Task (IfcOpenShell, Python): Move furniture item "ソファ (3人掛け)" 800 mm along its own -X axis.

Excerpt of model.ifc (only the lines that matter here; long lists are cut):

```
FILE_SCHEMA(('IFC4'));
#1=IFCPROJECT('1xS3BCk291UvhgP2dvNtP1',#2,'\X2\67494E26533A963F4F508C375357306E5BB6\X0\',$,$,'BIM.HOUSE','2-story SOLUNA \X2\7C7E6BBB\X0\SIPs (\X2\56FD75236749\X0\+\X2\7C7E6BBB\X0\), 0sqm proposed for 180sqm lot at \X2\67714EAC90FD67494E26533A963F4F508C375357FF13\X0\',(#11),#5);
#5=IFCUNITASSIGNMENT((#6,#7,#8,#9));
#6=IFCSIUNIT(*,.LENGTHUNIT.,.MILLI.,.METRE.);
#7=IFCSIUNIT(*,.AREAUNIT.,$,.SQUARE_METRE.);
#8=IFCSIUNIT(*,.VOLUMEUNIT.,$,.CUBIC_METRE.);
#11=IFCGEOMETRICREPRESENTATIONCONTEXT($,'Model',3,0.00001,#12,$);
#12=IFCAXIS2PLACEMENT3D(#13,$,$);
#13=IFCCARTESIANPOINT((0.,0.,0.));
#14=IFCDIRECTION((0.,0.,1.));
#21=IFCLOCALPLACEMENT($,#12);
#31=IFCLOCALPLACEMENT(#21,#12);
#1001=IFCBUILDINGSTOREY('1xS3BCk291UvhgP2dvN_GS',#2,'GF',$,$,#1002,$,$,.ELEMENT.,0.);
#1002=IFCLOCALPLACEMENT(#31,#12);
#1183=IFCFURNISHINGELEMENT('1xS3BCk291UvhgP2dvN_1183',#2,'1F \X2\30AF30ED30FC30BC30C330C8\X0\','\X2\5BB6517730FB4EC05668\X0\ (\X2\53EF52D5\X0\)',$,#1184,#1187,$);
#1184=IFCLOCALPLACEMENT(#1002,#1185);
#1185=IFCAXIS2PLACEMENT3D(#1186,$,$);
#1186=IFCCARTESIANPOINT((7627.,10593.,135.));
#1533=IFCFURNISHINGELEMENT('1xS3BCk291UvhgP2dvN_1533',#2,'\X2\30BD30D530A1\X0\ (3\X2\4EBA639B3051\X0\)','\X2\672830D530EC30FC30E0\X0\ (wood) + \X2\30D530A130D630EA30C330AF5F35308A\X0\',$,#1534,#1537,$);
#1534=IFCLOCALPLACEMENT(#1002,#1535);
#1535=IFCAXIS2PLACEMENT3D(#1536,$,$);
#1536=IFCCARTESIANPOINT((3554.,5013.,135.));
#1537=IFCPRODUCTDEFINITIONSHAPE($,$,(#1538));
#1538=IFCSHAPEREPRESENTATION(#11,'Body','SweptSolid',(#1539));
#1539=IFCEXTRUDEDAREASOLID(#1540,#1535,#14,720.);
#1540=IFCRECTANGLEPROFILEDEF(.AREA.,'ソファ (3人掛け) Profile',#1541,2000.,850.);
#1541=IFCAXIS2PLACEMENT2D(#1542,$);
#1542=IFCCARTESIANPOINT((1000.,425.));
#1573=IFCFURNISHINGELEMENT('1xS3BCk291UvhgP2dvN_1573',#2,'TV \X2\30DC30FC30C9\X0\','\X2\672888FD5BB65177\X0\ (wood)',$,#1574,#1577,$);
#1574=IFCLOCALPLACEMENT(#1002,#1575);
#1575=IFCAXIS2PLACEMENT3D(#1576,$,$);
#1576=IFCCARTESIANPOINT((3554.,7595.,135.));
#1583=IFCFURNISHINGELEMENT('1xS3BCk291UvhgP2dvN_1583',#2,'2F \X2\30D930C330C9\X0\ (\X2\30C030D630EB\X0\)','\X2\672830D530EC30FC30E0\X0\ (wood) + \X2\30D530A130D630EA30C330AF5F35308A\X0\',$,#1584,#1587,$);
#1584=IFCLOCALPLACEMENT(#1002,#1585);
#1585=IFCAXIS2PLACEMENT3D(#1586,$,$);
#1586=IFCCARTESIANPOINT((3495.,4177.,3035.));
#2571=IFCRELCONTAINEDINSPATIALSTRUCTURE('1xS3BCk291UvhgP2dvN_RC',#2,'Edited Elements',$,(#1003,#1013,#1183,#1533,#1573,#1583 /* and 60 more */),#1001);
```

```python
import ifcopenshell
import ifcopenshell.api.geometry
import ifcopenshell.util.placement
import ifcopenshell.util.unit

model = ifcopenshell.open("model.ifc")
unit_scale = ifcopenshell.util.unit.calculate_unit_scale(model)

item = model.by_guid("1xS3BCk291UvhgP2dvN_1533")
matrix = ifcopenshell.util.placement.get_local_placement(item.ObjectPlacement)
matrix[:3, 3] -= matrix[:3, 0] * 0.8 / unit_scale
ifcopenshell.api.geometry.edit_object_placement(model, product=item, matrix=matrix, is_si=False)

print(ifcopenshell.util.placement.get_local_placement(item.ObjectPlacement).round(3) + 0.0)

model.write("model_rev.ifc")
```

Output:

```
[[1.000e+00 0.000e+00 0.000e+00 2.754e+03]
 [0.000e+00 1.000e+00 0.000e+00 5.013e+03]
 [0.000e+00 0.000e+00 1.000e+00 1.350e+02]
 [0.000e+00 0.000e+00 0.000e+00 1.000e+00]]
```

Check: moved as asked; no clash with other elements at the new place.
